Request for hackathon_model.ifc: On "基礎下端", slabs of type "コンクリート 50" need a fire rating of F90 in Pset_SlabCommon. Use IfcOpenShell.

First a look at what the model holds.

```python
import ifcopenshell
import ifcopenshell.util.element

model = ifcopenshell.open("hackathon_model.ifc")
print(model.schema)
storey = next(s for s in model.by_type("IfcBuildingStorey") if s.Name == "基礎下端")
slabs = [e for e in ifcopenshell.util.element.get_decomposition(storey) if e.is_a("IfcSlab")]
seen = {}
for e in slabs:
    element_type = ifcopenshell.util.element.get_type(e)
    key = (element_type.Name if element_type != e and element_type else None, ifcopenshell.util.element.get_pset(e, "Pset_SlabCommon", "FireRating"))
    seen[key] = seen.get(key, 0) + 1
for (name, value), count in sorted(seen.items(), key=str):
    print(count, "x", name, "|", value)
```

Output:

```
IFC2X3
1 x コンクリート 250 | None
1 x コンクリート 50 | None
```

```python
import ifcopenshell
import ifcopenshell.api.pset
import ifcopenshell.util.element

model = ifcopenshell.open("hackathon_model.ifc")

storey = next(s for s in model.by_type("IfcBuildingStorey") if s.Name == "基礎下端")
slabs = [e for e in ifcopenshell.util.element.get_decomposition(storey) if e.is_a("IfcSlab")]

count = 0
for e in slabs:
    element_type = ifcopenshell.util.element.get_type(e)
    if element_type in (None, e) or element_type.Name != "コンクリート 50":
        continue
    # add_pset returns the element's existing set when there is one.
    pset = ifcopenshell.api.pset.add_pset(model, product=e, name="Pset_SlabCommon")
    ifcopenshell.api.pset.edit_pset(model, pset=pset, properties={"FireRating": "F90"})
    count += 1

print(count, "slabs updated")

model.write("hackathon_model-out.ifc")
```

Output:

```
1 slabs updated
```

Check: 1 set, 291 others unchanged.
